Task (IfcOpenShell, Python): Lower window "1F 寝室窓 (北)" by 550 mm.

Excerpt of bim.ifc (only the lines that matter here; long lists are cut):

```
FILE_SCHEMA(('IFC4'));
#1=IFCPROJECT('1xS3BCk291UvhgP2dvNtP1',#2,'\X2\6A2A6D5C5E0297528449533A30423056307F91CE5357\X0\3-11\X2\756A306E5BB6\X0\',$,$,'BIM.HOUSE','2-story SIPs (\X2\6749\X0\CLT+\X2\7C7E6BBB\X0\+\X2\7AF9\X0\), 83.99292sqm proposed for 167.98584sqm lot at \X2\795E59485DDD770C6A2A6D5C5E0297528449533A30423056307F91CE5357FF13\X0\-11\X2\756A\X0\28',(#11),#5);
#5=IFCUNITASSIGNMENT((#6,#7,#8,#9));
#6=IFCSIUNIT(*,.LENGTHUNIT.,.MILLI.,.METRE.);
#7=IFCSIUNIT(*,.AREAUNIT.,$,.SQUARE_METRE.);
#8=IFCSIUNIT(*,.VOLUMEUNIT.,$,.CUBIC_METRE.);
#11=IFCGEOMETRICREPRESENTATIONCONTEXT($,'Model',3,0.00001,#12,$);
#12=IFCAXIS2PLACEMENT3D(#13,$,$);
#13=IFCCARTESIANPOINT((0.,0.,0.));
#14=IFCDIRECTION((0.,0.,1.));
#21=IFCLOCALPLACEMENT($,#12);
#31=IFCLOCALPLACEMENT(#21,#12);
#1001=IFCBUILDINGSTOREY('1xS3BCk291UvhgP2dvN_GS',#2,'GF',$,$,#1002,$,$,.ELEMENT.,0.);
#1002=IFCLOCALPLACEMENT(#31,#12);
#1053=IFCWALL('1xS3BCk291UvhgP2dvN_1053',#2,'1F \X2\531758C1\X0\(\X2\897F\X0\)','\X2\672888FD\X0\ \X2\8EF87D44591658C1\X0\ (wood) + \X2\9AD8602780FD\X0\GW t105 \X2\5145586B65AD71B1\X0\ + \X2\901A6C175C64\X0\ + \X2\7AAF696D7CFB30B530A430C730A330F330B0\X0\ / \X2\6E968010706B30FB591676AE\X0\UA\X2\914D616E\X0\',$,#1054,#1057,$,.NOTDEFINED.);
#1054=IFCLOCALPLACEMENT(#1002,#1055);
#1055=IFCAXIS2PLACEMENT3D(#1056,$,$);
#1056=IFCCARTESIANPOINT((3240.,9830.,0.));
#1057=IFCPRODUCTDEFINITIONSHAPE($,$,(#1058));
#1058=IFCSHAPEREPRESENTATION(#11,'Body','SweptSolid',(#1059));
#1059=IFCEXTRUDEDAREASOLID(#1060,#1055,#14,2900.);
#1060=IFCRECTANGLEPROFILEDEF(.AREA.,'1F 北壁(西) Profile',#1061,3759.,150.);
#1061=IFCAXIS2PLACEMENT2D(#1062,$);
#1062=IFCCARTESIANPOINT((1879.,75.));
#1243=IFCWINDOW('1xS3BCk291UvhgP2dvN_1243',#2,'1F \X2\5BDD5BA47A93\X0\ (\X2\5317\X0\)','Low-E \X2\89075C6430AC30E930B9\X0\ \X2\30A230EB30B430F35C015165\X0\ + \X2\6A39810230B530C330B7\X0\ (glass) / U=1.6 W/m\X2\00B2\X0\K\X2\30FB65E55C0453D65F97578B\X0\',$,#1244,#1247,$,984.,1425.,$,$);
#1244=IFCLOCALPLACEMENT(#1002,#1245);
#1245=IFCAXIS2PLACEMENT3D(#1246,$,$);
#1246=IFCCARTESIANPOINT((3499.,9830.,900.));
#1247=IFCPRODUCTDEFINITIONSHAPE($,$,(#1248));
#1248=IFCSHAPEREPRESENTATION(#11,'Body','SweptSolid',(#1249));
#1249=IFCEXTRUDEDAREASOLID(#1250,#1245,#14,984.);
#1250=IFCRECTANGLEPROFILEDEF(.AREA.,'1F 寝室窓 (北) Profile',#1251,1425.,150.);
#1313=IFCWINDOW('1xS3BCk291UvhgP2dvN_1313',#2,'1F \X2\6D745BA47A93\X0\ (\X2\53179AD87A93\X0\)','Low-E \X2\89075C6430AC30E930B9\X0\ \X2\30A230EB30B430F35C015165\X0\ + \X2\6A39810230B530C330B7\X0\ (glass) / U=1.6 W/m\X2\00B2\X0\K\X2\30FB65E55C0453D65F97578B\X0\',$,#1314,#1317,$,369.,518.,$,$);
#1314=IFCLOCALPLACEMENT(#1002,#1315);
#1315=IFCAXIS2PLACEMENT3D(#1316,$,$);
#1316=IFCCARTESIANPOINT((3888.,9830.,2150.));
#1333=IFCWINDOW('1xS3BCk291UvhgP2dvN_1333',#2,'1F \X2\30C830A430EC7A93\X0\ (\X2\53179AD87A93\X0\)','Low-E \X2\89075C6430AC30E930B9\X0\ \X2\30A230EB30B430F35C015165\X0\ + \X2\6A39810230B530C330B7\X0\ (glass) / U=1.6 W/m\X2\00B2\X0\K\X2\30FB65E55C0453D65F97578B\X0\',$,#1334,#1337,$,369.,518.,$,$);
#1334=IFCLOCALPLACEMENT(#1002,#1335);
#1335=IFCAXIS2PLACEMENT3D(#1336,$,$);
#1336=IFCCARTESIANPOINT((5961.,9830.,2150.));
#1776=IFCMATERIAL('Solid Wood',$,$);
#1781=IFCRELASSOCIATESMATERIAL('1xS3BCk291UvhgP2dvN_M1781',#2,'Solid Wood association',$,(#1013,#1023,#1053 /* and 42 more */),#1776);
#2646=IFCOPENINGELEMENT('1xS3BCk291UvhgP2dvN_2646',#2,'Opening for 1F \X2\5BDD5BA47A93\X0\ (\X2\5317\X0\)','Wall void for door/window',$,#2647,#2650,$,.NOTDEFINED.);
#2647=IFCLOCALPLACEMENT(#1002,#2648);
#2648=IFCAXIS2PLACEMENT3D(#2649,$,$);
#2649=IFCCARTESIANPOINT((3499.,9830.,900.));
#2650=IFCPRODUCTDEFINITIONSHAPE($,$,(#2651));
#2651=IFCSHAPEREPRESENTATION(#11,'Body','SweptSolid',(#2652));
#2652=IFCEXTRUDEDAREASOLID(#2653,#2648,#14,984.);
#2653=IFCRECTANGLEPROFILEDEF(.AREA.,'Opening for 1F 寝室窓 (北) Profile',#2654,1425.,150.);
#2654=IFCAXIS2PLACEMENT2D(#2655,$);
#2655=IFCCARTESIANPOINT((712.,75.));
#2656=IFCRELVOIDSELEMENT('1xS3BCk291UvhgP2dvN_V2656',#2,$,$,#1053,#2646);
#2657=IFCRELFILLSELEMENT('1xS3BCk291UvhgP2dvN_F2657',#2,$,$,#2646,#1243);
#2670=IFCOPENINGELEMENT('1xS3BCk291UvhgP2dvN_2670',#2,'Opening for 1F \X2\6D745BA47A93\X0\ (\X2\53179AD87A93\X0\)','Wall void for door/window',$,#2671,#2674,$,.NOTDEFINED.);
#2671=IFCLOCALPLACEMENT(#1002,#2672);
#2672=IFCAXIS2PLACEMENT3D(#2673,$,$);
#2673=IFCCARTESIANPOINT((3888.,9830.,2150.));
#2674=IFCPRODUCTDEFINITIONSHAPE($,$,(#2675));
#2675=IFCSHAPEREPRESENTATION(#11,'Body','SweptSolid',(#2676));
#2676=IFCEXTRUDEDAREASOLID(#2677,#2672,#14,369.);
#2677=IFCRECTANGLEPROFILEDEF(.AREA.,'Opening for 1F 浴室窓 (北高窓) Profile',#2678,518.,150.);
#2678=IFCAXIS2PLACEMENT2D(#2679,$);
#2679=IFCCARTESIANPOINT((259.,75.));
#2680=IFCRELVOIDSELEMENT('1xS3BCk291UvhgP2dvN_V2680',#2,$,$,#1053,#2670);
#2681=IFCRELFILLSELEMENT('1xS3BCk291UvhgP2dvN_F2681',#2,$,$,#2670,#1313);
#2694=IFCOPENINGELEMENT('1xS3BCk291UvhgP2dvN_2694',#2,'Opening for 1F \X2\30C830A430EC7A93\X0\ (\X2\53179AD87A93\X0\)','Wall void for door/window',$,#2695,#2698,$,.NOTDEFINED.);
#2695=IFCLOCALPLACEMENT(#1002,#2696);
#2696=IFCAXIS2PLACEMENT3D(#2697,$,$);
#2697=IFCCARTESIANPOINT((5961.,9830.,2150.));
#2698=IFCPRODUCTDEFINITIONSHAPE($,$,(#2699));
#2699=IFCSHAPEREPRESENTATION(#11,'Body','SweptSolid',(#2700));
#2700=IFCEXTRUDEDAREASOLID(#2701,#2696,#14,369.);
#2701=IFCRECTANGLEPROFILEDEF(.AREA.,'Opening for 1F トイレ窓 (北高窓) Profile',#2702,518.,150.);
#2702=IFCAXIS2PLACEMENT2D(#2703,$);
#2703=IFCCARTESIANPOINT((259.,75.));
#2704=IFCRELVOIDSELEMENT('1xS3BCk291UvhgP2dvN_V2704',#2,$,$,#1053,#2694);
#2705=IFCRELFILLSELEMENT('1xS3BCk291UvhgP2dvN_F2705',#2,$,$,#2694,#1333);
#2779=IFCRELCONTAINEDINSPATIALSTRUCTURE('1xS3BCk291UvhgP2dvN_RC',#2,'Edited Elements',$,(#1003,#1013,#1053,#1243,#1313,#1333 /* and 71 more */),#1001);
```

```python
import numpy as np
import ifcopenshell
import ifcopenshell.api.geometry
import ifcopenshell.util.placement
import ifcopenshell.util.unit

model = ifcopenshell.open("bim.ifc")
unit_scale = ifcopenshell.util.unit.calculate_unit_scale(model)

window = model.by_id(1243)
opening = window.FillsVoids[0].RelatingOpeningElement
dz = -550.0

shift = np.array([0.0, 0.0, dz])
# The window is not placed relative to its opening, so move both.
for product in (opening, window):
    matrix = ifcopenshell.util.placement.get_local_placement(product.ObjectPlacement)
    matrix[:3, 3] += shift
    ifcopenshell.api.geometry.edit_object_placement(model, product=product, matrix=matrix, is_si=False)

print(f"moved by {dz * unit_scale:+.3f} m")

model.write("bim_rev.ifc")
```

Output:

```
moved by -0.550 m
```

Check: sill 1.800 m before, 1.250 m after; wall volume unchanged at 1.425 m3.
